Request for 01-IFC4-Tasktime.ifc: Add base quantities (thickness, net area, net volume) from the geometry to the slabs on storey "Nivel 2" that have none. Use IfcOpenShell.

First a look at what the model holds.

```python
import ifcopenshell
import ifcopenshell.util.element
import ifcopenshell.util.unit

model = ifcopenshell.open("01-IFC4-Tasktime.ifc")
print(model.schema)
for unit_type in ("LENGTHUNIT", "AREAUNIT", "VOLUMEUNIT"):
    print(unit_type, ifcopenshell.util.unit.calculate_unit_scale(model, unit_type))
storey = next(s for s in model.by_type("IfcBuildingStorey") if s.Name == "Nivel 2")
slabs = [e for e in ifcopenshell.util.element.get_decomposition(storey) if e.is_a("IfcSlab")]
for e in sorted(slabs, key=lambda e: e.id()):
    print(e.id(), e.is_a(), e.Name, list(ifcopenshell.util.element.get_psets(e, qtos_only=True)), sep=" | ")
```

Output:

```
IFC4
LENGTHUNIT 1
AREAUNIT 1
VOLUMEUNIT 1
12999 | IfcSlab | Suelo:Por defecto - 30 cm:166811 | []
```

```python
import ifcopenshell
import ifcopenshell.api.pset
import ifcopenshell.geom
import ifcopenshell.util.element
import ifcopenshell.util.shape
import ifcopenshell.util.unit

model = ifcopenshell.open("01-IFC4-Tasktime.ifc")
unit_scale = ifcopenshell.util.unit.calculate_unit_scale(model)
area_scale = ifcopenshell.util.unit.calculate_unit_scale(model, "AREAUNIT")
volume_scale = ifcopenshell.util.unit.calculate_unit_scale(model, "VOLUMEUNIT")
settings = ifcopenshell.geom.settings()

storey = next(s for s in model.by_type("IfcBuildingStorey") if s.Name == "Nivel 2")
slabs = [e for e in ifcopenshell.util.element.get_decomposition(storey) if e.is_a("IfcSlab")]

for e in sorted(slabs, key=lambda e: e.id()):
    if ifcopenshell.util.element.get_psets(e, qtos_only=True, should_inherit=False):
        continue
    # Geometry comes back in metres, in the element's own axes.
    shape = ifcopenshell.geom.create_shape(settings, e)
    values = {
        "Width": ifcopenshell.util.shape.get_z(shape.geometry) / unit_scale,
        "NetArea": ifcopenshell.util.shape.get_footprint_area(shape.geometry) / area_scale,
        "NetVolume": ifcopenshell.util.shape.get_volume(shape.geometry) / volume_scale,
    }
    qto = ifcopenshell.api.pset.add_qto(model, product=e, name="Qto_SlabBaseQuantities")
    ifcopenshell.api.pset.edit_qto(model, qto=qto, properties=values)
    print(e.id(), {k: round(v, 3) for k, v in values.items()})

model.write("01-IFC4-Tasktime-out.ifc")
```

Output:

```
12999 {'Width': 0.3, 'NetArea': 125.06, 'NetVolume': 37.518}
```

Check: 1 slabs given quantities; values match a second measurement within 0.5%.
